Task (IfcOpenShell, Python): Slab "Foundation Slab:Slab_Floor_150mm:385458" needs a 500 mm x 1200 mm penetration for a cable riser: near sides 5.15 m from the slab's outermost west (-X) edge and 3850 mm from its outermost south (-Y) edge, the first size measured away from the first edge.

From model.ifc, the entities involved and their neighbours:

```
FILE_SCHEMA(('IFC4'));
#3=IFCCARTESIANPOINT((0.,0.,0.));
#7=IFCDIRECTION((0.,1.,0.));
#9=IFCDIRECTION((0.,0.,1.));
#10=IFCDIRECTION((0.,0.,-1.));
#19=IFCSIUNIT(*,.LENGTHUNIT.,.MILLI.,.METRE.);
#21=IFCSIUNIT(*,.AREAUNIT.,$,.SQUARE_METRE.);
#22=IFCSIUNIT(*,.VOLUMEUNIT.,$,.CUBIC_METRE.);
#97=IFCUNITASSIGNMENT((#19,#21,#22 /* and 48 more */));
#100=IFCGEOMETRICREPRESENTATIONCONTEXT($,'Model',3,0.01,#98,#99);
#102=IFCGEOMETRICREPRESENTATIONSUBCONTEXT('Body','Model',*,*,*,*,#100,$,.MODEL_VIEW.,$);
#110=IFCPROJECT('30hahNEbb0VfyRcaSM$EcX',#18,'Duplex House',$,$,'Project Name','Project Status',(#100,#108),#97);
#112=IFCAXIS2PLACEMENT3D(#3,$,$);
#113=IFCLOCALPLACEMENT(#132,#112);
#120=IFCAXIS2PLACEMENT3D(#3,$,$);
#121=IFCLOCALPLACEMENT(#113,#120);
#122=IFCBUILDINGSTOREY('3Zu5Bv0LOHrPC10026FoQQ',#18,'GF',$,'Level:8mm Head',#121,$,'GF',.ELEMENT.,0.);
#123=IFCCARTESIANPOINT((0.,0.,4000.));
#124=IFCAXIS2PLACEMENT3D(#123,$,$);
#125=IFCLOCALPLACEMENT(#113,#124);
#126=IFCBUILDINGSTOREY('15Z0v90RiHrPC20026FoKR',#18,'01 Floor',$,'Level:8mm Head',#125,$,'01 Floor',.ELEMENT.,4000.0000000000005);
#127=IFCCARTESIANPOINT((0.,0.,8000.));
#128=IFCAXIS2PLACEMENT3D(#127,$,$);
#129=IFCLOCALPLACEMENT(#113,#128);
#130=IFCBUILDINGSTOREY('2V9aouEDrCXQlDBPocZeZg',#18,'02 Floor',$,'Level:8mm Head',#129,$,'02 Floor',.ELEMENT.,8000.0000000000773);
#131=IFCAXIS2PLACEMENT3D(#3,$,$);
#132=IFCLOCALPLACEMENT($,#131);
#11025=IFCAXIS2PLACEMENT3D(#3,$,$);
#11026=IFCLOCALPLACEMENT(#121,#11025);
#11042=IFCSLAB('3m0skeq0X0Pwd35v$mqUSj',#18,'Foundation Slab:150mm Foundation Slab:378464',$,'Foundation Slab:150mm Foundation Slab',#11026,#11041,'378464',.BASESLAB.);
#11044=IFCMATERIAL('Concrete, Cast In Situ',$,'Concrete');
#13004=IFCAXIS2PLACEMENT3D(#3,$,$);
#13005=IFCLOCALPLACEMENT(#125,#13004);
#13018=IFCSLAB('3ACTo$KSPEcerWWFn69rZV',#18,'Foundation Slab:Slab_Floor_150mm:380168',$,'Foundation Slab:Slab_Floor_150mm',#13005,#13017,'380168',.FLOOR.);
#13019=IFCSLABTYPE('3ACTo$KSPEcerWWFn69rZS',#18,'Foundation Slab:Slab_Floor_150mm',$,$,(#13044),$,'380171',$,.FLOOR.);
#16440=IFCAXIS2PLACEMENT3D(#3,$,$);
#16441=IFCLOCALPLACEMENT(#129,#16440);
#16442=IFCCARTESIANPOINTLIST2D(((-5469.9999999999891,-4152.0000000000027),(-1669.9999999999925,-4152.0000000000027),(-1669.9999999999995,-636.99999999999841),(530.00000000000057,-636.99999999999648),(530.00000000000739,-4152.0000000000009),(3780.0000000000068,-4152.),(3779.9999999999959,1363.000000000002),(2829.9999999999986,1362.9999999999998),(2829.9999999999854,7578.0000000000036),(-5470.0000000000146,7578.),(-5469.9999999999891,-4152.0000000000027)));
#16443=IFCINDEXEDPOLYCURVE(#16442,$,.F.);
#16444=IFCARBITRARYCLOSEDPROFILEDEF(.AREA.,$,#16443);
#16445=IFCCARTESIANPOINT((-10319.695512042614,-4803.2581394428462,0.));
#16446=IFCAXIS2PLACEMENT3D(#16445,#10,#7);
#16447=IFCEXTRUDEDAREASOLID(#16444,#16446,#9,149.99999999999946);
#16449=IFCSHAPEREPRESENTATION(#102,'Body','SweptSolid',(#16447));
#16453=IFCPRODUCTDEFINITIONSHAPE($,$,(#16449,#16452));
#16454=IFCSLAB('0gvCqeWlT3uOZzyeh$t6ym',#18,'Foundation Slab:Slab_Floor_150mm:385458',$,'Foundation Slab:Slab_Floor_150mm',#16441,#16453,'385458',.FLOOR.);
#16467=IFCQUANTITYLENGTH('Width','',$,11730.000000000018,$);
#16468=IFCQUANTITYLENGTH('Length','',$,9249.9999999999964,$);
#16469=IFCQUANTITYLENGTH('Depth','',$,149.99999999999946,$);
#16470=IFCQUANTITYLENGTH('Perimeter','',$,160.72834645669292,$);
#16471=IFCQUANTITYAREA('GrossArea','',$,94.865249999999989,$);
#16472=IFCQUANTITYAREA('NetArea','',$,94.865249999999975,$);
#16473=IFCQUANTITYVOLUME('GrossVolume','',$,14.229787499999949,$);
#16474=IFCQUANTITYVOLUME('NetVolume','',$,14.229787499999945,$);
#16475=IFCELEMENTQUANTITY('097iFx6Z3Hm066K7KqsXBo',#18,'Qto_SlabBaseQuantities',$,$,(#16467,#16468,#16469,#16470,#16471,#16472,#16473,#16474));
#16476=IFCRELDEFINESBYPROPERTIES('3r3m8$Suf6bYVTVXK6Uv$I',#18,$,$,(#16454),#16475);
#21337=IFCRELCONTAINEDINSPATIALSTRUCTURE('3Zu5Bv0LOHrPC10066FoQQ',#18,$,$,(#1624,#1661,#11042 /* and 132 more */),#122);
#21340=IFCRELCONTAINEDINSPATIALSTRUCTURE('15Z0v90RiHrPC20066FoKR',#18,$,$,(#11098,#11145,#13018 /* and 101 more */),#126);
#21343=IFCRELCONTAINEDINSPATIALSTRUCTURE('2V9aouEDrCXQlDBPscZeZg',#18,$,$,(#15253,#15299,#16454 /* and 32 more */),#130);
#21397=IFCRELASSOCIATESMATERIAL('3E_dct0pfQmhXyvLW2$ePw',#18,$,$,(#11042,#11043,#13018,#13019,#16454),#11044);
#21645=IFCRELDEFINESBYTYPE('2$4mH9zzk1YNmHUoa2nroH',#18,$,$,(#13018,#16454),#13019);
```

```python
import numpy as np
import ifcopenshell
import ifcopenshell.api.feature
import ifcopenshell.api.geometry
import ifcopenshell.api.pset
import ifcopenshell.api.root
import ifcopenshell.geom
import ifcopenshell.util.element
import ifcopenshell.util.placement
import ifcopenshell.util.representation
import ifcopenshell.util.shape
import ifcopenshell.util.unit

model = ifcopenshell.open("model.ifc")
unit_scale = ifcopenshell.util.unit.calculate_unit_scale(model)
area_scale = ifcopenshell.util.unit.calculate_unit_scale(model, "AREAUNIT")
volume_scale = ifcopenshell.util.unit.calculate_unit_scale(model, "VOLUMEUNIT")
settings = ifcopenshell.geom.settings()


def volume(element):
    """Net volume in cubic metres, openings subtracted."""
    shape = ifcopenshell.geom.create_shape(settings, element)
    return ifcopenshell.util.shape.get_volume(shape.geometry)


slab = model.by_guid("0gvCqeWlT3uOZzyeh$t6ym")
before = volume(slab)

# Extent in the slab's own axes, in metres. The edges named are its -X and -Y sides.
slab_shape = ifcopenshell.geom.create_shape(settings, slab)
vertices = ifcopenshell.util.shape.get_vertices(slab_shape.geometry)
x_min, y_min, bottom = vertices.min(axis=0)
top = vertices[:, 2].max()

opening = ifcopenshell.api.root.create_entity(model, ifc_class="IfcOpeningElement", name="Cable riser opening", predefined_type="OPENING")
context = ifcopenshell.util.representation.get_context(model, "Model", "Body", "MODEL_VIEW")
width, depth = 0.5, 1.2
outline = [(0.0, 0.0), (width, 0.0), (width, depth), (0.0, depth), (0.0, 0.0)]
# Overshoot both faces by 50 mm so the cut is clean.
shape = ifcopenshell.api.geometry.add_slab_representation(
    model, context=context, depth=top - bottom + 0.1, polyline=outline
)
ifcopenshell.api.geometry.assign_representation(model, product=opening, representation=shape)

matrix = ifcopenshell.util.placement.get_local_placement(slab.ObjectPlacement)
matrix[:, 3] = matrix @ np.append(np.array([x_min + 5.15, y_min + 3.85, bottom - 0.05]) / unit_scale, 1.0)
ifcopenshell.api.geometry.edit_object_placement(model, product=opening, matrix=matrix, is_si=False)
ifcopenshell.api.feature.add_feature(model, feature=opening, element=slab)

after = volume(slab)

# Update the slab's stored quantities.
qto = model.by_id(ifcopenshell.util.element.get_pset(slab, "Qto_SlabBaseQuantities", should_inherit=False)["id"])
ifcopenshell.api.pset.edit_qto(model, qto=qto, properties={
    "NetArea": after / (top - bottom) / area_scale,
    "NetVolume": after / volume_scale,
})

print(f"slab volume {before:.3f} -> {after:.3f} m3")

model.write("model_v2.ifc")
```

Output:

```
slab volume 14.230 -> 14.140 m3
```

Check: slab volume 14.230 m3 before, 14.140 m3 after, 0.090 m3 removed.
